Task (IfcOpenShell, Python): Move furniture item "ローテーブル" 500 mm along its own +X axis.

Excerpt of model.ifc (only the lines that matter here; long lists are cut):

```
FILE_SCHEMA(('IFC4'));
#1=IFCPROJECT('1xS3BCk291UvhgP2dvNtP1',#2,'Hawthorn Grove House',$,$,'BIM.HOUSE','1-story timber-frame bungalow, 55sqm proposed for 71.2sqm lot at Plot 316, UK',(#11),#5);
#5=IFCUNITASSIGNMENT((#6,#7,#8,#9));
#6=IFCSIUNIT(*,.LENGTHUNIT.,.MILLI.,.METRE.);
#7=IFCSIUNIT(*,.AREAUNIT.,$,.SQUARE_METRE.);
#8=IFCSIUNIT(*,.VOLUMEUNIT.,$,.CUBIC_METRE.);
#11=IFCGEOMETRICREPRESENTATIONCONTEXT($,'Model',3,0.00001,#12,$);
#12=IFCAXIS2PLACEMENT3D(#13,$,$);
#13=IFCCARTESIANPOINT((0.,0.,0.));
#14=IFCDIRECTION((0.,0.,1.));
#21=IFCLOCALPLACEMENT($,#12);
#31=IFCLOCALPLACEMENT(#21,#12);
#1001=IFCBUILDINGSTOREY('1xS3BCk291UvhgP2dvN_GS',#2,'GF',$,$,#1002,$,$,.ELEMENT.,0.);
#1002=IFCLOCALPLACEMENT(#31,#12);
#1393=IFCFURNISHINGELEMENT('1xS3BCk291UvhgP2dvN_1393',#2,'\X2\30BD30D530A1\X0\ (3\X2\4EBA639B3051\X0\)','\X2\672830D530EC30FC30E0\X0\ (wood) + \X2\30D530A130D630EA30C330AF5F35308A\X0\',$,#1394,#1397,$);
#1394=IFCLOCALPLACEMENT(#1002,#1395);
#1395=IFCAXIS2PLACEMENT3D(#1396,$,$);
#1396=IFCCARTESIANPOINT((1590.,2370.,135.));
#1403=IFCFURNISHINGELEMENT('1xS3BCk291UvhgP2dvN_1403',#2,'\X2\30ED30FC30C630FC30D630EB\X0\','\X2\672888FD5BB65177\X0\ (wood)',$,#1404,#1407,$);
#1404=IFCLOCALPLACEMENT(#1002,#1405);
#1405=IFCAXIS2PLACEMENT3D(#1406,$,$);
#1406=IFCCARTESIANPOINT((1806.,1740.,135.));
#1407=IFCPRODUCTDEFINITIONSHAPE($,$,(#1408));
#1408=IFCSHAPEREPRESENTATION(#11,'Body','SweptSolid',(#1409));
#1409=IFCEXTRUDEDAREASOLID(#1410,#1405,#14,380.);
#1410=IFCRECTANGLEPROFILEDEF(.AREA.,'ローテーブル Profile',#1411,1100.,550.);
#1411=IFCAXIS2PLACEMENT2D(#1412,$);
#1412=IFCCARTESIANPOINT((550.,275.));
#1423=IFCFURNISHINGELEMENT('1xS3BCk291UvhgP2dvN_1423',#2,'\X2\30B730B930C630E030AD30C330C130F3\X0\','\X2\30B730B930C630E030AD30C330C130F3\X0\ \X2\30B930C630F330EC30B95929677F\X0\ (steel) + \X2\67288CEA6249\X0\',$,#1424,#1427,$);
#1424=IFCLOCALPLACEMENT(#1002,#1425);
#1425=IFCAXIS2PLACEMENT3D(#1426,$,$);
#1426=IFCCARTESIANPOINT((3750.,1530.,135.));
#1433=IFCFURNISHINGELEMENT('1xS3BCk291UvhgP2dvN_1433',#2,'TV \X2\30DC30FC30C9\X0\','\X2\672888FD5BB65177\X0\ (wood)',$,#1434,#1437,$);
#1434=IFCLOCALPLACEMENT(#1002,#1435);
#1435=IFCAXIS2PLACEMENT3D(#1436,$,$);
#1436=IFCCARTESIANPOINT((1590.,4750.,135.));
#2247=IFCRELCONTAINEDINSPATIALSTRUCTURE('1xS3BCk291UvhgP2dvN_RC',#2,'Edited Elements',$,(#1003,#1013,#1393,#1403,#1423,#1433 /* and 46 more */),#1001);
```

```python
import ifcopenshell
import ifcopenshell.api.geometry
import ifcopenshell.util.placement
import ifcopenshell.util.unit

model = ifcopenshell.open("model.ifc")
unit_scale = ifcopenshell.util.unit.calculate_unit_scale(model)

item = model.by_guid("1xS3BCk291UvhgP2dvN_1403")
matrix = ifcopenshell.util.placement.get_local_placement(item.ObjectPlacement)
matrix[:3, 3] += matrix[:3, 0] * 0.5 / unit_scale
ifcopenshell.api.geometry.edit_object_placement(model, product=item, matrix=matrix, is_si=False)

print(ifcopenshell.util.placement.get_local_placement(item.ObjectPlacement).round(3) + 0.0)

model.write("model-out.ifc")
```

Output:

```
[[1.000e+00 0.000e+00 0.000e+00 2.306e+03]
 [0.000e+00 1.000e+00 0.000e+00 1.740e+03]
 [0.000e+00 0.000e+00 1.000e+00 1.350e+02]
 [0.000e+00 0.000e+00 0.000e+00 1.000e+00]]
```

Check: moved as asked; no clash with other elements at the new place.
